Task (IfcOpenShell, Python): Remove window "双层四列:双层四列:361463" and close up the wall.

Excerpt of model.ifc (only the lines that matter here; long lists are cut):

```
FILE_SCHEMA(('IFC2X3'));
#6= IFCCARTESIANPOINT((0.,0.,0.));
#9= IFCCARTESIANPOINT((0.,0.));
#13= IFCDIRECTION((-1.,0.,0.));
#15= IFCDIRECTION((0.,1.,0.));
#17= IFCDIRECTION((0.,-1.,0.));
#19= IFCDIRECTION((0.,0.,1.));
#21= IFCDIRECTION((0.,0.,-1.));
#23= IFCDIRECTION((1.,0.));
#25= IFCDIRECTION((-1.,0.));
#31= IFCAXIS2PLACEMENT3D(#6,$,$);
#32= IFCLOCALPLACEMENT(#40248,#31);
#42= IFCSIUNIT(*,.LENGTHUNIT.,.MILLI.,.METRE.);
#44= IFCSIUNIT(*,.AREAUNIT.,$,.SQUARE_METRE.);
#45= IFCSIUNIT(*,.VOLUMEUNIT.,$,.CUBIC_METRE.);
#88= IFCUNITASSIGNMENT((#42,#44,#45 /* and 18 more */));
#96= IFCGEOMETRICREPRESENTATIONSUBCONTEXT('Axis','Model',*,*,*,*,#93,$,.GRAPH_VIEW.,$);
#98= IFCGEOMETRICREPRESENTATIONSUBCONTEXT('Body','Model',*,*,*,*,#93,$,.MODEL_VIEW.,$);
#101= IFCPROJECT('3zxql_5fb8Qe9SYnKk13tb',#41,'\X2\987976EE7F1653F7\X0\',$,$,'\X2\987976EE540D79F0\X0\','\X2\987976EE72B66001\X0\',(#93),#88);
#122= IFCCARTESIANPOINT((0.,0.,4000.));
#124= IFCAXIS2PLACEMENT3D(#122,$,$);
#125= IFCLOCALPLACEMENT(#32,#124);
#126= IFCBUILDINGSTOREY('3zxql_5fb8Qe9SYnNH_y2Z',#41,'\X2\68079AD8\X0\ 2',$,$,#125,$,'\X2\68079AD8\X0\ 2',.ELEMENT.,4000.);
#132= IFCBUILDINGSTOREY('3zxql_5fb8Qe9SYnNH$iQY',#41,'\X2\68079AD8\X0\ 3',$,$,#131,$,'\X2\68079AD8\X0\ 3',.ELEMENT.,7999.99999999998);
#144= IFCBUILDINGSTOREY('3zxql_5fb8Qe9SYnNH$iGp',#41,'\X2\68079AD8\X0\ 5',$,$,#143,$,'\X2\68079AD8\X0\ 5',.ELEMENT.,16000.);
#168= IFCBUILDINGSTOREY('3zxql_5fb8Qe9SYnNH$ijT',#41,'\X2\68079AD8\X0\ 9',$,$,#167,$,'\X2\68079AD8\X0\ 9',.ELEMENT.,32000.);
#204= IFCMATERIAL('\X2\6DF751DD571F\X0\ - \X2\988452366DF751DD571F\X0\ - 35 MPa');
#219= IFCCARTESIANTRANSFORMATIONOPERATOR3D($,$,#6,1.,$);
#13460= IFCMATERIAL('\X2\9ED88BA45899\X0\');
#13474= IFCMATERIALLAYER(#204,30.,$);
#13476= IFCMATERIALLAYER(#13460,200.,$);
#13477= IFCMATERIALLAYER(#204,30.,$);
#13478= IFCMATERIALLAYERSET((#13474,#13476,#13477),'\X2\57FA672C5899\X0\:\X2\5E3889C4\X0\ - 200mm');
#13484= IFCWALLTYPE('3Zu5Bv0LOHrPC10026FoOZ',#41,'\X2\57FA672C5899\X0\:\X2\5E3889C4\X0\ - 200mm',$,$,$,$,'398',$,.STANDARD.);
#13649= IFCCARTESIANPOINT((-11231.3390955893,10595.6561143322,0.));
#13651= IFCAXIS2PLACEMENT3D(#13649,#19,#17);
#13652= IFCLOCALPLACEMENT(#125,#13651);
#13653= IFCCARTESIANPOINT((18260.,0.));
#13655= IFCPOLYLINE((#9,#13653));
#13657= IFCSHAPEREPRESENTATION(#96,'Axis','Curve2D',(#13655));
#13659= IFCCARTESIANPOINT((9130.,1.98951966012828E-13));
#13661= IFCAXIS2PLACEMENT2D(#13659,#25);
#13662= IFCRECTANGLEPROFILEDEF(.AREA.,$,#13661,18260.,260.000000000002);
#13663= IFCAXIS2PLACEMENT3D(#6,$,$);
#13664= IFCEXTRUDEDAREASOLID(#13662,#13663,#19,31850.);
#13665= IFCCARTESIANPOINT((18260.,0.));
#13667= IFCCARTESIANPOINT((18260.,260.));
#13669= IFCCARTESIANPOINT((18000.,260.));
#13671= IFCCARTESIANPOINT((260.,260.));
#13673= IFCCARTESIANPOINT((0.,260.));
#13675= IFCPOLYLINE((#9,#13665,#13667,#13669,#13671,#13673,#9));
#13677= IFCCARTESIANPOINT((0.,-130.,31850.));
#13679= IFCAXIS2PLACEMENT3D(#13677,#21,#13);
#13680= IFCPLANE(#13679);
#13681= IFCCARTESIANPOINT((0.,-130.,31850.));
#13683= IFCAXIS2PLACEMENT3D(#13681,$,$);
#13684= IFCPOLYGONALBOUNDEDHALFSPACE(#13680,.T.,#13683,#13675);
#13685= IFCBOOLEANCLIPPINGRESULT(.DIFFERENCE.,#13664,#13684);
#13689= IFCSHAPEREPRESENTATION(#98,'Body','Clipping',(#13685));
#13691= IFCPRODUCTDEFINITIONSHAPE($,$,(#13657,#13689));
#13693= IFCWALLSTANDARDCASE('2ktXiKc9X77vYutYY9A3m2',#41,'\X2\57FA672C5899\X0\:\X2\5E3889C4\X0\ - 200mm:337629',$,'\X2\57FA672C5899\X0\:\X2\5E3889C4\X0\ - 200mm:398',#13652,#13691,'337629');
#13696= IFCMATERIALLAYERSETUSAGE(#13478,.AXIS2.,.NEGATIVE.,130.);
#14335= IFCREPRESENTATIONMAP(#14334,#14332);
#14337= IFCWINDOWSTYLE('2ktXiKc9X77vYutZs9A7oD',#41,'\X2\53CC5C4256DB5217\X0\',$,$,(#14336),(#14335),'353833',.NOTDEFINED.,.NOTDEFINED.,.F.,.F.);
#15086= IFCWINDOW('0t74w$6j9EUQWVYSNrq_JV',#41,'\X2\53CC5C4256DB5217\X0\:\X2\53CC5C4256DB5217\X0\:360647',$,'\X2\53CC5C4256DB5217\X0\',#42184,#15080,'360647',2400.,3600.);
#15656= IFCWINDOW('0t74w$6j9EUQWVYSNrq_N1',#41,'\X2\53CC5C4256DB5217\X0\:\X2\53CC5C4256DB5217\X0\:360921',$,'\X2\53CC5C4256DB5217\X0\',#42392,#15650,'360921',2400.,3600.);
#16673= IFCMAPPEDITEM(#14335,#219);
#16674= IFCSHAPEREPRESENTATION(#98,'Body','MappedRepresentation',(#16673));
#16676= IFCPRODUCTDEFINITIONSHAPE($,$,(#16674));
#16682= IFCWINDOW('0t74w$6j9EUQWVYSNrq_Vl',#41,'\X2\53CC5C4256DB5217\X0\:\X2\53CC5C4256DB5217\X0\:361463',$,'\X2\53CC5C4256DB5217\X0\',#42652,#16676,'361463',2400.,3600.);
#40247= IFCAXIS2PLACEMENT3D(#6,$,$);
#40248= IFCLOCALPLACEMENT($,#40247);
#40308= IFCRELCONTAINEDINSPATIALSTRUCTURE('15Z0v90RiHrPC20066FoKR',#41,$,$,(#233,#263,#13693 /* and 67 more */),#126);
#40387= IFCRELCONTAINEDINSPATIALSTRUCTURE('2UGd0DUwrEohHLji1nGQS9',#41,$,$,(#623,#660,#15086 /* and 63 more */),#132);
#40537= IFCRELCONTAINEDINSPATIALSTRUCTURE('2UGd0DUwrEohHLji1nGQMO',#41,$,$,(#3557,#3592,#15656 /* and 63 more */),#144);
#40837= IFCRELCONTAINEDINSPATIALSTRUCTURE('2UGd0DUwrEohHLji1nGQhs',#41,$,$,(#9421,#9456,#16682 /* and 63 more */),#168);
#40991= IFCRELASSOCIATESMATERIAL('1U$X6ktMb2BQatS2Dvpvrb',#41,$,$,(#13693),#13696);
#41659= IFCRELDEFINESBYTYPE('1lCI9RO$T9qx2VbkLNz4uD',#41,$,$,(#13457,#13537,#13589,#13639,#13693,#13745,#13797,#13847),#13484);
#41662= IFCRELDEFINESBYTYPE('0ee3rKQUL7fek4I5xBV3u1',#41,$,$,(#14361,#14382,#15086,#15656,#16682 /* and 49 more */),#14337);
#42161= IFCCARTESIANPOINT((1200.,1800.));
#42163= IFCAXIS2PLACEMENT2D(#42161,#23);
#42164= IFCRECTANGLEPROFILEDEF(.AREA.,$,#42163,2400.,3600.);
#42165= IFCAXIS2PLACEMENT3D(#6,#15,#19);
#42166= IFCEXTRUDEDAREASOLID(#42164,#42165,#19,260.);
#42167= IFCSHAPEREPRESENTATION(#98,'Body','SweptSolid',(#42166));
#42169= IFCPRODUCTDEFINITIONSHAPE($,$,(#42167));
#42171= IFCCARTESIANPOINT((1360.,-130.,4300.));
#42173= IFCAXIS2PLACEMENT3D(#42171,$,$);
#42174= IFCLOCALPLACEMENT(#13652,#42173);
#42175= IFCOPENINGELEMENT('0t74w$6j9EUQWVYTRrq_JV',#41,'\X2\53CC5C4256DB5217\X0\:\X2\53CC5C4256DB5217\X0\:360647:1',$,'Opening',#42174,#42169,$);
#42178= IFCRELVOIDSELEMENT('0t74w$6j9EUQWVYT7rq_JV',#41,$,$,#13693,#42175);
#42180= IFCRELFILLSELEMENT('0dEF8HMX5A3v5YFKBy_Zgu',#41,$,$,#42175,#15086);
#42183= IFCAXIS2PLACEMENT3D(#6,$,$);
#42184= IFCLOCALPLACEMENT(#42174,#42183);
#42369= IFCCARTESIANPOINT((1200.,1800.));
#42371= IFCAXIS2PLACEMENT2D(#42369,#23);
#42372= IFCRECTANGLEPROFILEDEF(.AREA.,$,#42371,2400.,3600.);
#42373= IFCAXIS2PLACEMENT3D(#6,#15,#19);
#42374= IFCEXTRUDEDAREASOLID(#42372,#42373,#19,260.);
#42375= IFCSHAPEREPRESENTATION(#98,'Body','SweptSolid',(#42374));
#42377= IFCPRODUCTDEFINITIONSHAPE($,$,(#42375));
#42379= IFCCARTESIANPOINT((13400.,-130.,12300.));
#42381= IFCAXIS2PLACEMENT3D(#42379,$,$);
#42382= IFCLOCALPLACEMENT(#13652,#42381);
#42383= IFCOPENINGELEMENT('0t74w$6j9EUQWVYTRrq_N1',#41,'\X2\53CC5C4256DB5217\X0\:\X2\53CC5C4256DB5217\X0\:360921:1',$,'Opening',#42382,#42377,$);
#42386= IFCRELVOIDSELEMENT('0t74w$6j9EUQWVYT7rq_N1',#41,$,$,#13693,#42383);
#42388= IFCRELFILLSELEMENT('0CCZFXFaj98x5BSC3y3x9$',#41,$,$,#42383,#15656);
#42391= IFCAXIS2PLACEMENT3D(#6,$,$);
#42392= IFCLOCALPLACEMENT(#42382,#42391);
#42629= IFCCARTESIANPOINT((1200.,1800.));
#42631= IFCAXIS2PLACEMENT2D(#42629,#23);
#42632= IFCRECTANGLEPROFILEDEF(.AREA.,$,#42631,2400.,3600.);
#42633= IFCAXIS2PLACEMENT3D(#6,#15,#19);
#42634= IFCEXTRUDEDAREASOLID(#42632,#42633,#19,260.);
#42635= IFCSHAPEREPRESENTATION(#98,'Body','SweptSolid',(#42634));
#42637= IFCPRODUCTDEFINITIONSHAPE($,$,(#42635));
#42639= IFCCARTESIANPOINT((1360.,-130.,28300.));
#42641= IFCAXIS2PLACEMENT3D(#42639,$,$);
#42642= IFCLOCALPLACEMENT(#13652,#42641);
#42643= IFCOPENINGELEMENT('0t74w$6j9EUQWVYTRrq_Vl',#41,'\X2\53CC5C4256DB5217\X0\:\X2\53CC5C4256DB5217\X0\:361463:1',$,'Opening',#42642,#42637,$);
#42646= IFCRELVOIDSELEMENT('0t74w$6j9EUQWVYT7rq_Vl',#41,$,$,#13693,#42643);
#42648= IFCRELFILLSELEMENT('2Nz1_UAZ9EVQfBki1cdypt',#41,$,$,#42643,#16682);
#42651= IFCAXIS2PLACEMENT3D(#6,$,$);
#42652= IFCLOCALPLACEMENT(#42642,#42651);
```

```python
import ifcopenshell
import ifcopenshell.api.feature
import ifcopenshell.api.root
import ifcopenshell.geom
import ifcopenshell.util.shape

model = ifcopenshell.open("model.ifc")
settings = ifcopenshell.geom.settings()


def volume(element):
    """Net volume in cubic metres, openings subtracted."""
    shape = ifcopenshell.geom.create_shape(settings, element)
    return ifcopenshell.util.shape.get_volume(shape.geometry)


window = model.by_guid("0t74w$6j9EUQWVYSNrq_Vl")
opening = window.FillsVoids[0].RelatingOpeningElement
wall = opening.VoidsElements[0].RelatingBuildingElement
before = volume(wall)

ifcopenshell.api.root.remove_product(model, product=window)
ifcopenshell.api.feature.remove_feature(model, feature=opening)

after = volume(wall)

print(f"wall volume {before:.3f} -> {after:.3f} m3")

model.write("model-out.ifc")
```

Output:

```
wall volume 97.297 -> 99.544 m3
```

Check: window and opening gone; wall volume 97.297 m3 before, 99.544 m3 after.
